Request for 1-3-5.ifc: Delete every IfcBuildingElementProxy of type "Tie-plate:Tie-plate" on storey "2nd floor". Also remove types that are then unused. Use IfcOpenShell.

First a look at what the model holds.

```python
import ifcopenshell
import ifcopenshell.util.element

model = ifcopenshell.open("1-3-5.ifc")
print(model.schema)
storey = next(s for s in model.by_type("IfcBuildingStorey") if s.Name == "2nd floor")
proxies = [e for e in ifcopenshell.util.element.get_decomposition(storey) if e.is_a("IfcBuildingElementProxy")]
seen = {}
for e in proxies:
    element_type = ifcopenshell.util.element.get_type(e)
    name = element_type.Name if element_type not in (None, e) else None
    seen[name] = seen.get(name, 0) + 1
for name, count in sorted(seen.items(), key=str):
    print(count, "x", name)
```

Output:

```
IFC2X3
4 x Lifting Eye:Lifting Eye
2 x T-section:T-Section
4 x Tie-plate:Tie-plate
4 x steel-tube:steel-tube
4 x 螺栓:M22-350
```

```python
import ifcopenshell
import ifcopenshell.api.root
import ifcopenshell.util.element

model = ifcopenshell.open("1-3-5.ifc")

storey = next(s for s in model.by_type("IfcBuildingStorey") if s.Name == "2nd floor")
proxies = [e for e in ifcopenshell.util.element.get_decomposition(storey) if e.is_a("IfcBuildingElementProxy")]
targets = [e for e in proxies if (t := ifcopenshell.util.element.get_type(e)) not in (None, e) and t.Name == "Tie-plate:Tie-plate"]
types = {ifcopenshell.util.element.get_type(e) for e in targets} - {None, *targets}

for e in targets:
    ifcopenshell.api.root.remove_product(model, product=e)
print(len(targets), "removed")

unused = [t for t in types if not ifcopenshell.util.element.get_types(t)]
for t in unused:
    ifcopenshell.api.root.remove_product(model, product=t)
print(len(unused), "unused types removed")

model.write("1-3-5_v2.ifc")
```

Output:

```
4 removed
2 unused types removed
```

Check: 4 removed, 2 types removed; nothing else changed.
